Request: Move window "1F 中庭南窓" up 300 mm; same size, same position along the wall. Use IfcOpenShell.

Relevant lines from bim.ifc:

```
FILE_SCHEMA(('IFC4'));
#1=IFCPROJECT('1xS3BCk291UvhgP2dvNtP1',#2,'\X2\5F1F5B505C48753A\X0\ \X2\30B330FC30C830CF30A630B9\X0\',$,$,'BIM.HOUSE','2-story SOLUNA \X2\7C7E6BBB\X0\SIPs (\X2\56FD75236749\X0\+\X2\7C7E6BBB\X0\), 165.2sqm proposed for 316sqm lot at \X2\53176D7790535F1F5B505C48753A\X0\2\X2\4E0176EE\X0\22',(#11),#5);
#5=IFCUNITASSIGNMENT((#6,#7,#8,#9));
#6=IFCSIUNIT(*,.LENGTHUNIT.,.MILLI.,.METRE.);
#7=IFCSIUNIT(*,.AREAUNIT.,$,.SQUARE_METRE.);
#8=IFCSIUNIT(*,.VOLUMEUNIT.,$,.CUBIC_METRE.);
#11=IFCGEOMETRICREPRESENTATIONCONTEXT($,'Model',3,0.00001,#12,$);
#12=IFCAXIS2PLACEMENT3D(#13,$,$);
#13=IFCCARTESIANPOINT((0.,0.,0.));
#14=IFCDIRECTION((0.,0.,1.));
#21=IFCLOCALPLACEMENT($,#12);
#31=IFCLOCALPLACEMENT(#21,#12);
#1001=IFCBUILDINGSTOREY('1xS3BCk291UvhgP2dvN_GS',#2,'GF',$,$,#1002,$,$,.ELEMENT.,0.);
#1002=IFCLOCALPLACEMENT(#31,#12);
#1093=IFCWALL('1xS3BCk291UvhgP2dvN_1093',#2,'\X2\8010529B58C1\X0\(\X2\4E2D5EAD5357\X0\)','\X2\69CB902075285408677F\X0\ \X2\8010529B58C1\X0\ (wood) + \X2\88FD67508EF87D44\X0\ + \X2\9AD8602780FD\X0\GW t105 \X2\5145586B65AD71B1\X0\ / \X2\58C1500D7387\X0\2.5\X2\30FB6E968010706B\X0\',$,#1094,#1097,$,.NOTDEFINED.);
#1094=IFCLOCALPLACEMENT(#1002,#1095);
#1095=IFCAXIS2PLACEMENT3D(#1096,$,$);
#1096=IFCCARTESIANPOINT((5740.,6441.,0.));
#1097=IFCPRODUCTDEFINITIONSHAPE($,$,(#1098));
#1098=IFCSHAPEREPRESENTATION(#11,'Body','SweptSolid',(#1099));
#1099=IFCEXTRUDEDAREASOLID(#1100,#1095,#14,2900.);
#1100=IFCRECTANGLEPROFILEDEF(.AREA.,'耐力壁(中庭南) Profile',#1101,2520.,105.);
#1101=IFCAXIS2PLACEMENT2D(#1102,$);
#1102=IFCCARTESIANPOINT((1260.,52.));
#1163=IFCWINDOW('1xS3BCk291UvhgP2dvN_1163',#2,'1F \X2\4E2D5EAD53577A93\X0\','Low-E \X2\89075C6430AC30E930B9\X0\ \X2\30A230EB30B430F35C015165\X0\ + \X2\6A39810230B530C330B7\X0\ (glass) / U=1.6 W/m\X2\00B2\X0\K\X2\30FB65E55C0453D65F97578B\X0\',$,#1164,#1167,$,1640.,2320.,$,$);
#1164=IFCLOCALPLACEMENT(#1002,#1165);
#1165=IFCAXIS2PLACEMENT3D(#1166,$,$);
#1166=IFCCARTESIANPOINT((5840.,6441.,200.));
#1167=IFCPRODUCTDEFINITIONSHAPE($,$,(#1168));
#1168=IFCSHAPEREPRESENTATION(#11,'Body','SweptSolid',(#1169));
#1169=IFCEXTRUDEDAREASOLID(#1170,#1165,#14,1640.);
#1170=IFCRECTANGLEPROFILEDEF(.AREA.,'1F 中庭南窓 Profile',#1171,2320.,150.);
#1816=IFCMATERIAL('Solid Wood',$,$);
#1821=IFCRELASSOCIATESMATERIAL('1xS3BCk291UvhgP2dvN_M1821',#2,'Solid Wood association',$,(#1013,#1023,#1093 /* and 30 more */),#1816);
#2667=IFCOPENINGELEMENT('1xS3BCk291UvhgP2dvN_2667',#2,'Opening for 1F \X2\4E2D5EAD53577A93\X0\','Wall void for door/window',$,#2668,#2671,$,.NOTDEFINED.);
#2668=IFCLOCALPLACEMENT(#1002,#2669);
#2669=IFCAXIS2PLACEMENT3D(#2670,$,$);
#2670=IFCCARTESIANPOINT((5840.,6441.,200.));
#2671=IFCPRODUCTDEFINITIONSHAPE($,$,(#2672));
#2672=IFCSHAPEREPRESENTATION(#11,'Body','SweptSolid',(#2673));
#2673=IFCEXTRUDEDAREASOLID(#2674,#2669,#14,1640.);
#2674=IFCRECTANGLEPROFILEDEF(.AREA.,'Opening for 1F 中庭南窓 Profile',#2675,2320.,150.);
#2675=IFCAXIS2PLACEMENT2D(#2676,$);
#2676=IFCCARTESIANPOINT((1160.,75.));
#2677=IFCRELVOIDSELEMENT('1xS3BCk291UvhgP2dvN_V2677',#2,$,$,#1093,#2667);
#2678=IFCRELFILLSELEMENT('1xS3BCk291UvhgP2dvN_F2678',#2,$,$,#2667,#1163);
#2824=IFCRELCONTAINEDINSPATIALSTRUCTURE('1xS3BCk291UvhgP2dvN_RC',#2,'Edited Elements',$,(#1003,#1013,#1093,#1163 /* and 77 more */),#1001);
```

```python
import numpy as np
import ifcopenshell
import ifcopenshell.api.geometry
import ifcopenshell.util.placement
import ifcopenshell.util.unit

model = ifcopenshell.open("bim.ifc")
unit_scale = ifcopenshell.util.unit.calculate_unit_scale(model)

window = model.by_guid("1xS3BCk291UvhgP2dvN_1163")
opening = window.FillsVoids[0].RelatingOpeningElement
dz = 0.3 / unit_scale

shift = np.array([0.0, 0.0, dz])
# The window is not placed relative to its opening, so move both.
for product in (opening, window):
    matrix = ifcopenshell.util.placement.get_local_placement(product.ObjectPlacement)
    matrix[:3, 3] += shift
    ifcopenshell.api.geometry.edit_object_placement(model, product=product, matrix=matrix, is_si=False)

print(f"moved by {dz * unit_scale:+.3f} m")

model.write("bim_v2.ifc")
```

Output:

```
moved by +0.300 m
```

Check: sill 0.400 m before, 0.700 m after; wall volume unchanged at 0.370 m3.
